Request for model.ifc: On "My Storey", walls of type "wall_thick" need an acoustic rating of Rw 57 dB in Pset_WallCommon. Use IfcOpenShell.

First a look at what the model holds.

```python
import ifcopenshell
import ifcopenshell.util.element

model = ifcopenshell.open("model.ifc")
print(model.schema)
storey = next(s for s in model.by_type("IfcBuildingStorey") if s.Name == "My Storey")
walls = [e for e in ifcopenshell.util.element.get_decomposition(storey) if e.is_a("IfcWall")]
seen = {}
for e in walls:
    element_type = ifcopenshell.util.element.get_type(e)
    key = (element_type.Name if element_type != e and element_type else None, ifcopenshell.util.element.get_pset(e, "Pset_WallCommon", "AcousticRating"))
    seen[key] = seen.get(key, 0) + 1
for (name, value), count in sorted(seen.items(), key=str):
    print(count, "x", name, "|", value)
```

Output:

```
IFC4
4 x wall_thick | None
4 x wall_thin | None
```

```python
import ifcopenshell
import ifcopenshell.api.pset
import ifcopenshell.util.element

model = ifcopenshell.open("model.ifc")

storey = next(s for s in model.by_type("IfcBuildingStorey") if s.Name == "My Storey")
walls = [e for e in ifcopenshell.util.element.get_decomposition(storey) if e.is_a("IfcWall")]

count = 0
for e in walls:
    element_type = ifcopenshell.util.element.get_type(e)
    if element_type in (None, e) or element_type.Name != "wall_thick":
        continue
    # add_pset returns the element's existing set when there is one.
    pset = ifcopenshell.api.pset.add_pset(model, product=e, name="Pset_WallCommon")
    ifcopenshell.api.pset.edit_pset(model, pset=pset, properties={"AcousticRating": "Rw 57 dB"})
    count += 1

print(count, "walls updated")

model.write("model_updated.ifc")
```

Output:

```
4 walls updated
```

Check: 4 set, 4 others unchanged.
